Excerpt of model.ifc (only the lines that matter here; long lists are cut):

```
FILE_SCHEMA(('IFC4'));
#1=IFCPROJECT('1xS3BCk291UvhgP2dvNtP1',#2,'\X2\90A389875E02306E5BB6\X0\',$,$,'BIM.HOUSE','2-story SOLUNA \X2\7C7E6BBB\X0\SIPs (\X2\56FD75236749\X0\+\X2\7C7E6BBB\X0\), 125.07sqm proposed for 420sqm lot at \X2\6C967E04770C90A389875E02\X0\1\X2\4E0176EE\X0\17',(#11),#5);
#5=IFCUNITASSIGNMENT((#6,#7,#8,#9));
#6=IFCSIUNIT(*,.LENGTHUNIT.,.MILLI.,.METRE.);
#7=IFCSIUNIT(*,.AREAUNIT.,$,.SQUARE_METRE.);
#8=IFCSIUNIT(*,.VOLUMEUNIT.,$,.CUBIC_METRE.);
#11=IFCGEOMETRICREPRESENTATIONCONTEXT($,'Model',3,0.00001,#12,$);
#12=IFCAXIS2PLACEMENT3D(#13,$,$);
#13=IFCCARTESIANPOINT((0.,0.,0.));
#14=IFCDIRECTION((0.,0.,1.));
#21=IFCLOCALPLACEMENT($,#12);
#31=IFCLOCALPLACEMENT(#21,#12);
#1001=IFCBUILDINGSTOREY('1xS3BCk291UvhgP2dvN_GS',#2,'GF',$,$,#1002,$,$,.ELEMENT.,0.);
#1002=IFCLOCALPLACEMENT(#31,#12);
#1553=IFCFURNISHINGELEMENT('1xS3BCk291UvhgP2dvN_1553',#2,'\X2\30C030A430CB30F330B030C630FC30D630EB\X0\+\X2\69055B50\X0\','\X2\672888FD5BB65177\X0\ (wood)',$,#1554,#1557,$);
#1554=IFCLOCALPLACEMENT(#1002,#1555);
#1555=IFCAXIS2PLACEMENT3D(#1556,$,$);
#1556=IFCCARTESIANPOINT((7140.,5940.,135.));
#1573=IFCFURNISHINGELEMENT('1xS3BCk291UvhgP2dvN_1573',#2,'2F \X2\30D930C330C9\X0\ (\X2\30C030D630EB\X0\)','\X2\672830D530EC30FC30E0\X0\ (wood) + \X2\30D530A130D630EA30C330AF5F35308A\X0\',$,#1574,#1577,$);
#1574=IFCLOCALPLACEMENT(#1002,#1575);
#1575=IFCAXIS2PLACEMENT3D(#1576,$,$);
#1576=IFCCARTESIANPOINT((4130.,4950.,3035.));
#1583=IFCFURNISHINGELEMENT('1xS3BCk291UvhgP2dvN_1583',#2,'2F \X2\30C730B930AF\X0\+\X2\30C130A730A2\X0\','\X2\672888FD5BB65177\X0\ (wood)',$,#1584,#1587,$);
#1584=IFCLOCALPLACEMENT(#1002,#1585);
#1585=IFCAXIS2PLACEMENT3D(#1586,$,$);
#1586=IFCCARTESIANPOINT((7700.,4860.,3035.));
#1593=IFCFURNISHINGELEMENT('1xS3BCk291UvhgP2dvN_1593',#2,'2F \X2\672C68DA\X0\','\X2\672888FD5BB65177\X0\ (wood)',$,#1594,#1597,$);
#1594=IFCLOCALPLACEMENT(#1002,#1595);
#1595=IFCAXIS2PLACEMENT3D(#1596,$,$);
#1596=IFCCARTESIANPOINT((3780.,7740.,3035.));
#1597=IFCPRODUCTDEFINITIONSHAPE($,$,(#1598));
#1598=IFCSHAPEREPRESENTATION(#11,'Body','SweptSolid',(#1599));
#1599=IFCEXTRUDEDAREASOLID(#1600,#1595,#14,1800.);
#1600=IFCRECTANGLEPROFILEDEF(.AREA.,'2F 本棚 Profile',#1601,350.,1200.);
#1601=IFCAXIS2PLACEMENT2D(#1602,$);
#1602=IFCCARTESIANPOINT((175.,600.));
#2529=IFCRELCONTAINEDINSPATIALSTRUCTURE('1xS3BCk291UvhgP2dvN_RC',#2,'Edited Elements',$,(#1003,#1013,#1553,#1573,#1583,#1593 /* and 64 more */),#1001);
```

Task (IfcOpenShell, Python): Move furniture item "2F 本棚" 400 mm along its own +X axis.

```python
import ifcopenshell
import ifcopenshell.api.geometry
import ifcopenshell.util.placement
import ifcopenshell.util.unit

model = ifcopenshell.open("model.ifc")
unit_scale = ifcopenshell.util.unit.calculate_unit_scale(model)

item = model.by_guid("1xS3BCk291UvhgP2dvN_1593")
matrix = ifcopenshell.util.placement.get_local_placement(item.ObjectPlacement)
matrix[:3, 3] += matrix[:3, 0] * 0.4 / unit_scale
ifcopenshell.api.geometry.edit_object_placement(model, product=item, matrix=matrix, is_si=False)

print(ifcopenshell.util.placement.get_local_placement(item.ObjectPlacement).round(3) + 0.0)

model.write("model_updated.ifc")
```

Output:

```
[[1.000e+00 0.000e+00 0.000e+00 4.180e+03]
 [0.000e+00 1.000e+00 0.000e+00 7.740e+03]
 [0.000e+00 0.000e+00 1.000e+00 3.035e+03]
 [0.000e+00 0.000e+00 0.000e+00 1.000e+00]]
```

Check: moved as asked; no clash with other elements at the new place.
